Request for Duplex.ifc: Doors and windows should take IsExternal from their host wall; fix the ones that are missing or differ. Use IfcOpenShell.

First a look at what the model holds.

```python
import ifcopenshell
import ifcopenshell.util.element

model = ifcopenshell.open("Duplex.ifc")
print(model.schema)
seen = {}
for e in model.by_type("IfcDoor") + model.by_type("IfcWindow"):
    if not e.FillsVoids:
        continue
    host = e.FillsVoids[0].RelatingOpeningElement.VoidsElements[0].RelatingBuildingElement
    own = ifcopenshell.util.element.get_pset(e, f"Pset_{e.is_a()[3:].removesuffix('StandardCase')}Common", "IsExternal")
    wall = ifcopenshell.util.element.get_pset(host, "Pset_WallCommon", "IsExternal")
    seen[e.is_a(), own, wall] = seen.get((e.is_a(), own, wall), 0) + 1
for (cls, own, wall), count in sorted(seen.items(), key=str):
    print(count, cls, "IsExternal:", own, "| host wall:", wall)
```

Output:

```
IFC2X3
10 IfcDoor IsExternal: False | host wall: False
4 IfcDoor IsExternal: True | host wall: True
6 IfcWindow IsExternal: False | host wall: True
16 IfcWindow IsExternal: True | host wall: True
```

```python
import ifcopenshell
import ifcopenshell.api.pset
import ifcopenshell.util.element

model = ifcopenshell.open("Duplex.ifc")

count = 0
for ifc_class, pset_name in (("IfcDoor", "Pset_DoorCommon"), ("IfcWindow", "Pset_WindowCommon")):
    for e in model.by_type(ifc_class):
        if not e.FillsVoids:
            continue
        host = e.FillsVoids[0].RelatingOpeningElement.VoidsElements[0].RelatingBuildingElement
        external = ifcopenshell.util.element.get_pset(host, "Pset_WallCommon", "IsExternal")
        if external is None or ifcopenshell.util.element.get_pset(e, pset_name, "IsExternal") == external:
            continue
        pset = ifcopenshell.api.pset.add_pset(model, product=e, name=pset_name)
        ifcopenshell.api.pset.edit_pset(model, pset=pset, properties={"IsExternal": external})
        count += 1

print(count, "updated")

model.write("Duplex_updated.ifc")
```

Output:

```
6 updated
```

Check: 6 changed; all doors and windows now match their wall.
